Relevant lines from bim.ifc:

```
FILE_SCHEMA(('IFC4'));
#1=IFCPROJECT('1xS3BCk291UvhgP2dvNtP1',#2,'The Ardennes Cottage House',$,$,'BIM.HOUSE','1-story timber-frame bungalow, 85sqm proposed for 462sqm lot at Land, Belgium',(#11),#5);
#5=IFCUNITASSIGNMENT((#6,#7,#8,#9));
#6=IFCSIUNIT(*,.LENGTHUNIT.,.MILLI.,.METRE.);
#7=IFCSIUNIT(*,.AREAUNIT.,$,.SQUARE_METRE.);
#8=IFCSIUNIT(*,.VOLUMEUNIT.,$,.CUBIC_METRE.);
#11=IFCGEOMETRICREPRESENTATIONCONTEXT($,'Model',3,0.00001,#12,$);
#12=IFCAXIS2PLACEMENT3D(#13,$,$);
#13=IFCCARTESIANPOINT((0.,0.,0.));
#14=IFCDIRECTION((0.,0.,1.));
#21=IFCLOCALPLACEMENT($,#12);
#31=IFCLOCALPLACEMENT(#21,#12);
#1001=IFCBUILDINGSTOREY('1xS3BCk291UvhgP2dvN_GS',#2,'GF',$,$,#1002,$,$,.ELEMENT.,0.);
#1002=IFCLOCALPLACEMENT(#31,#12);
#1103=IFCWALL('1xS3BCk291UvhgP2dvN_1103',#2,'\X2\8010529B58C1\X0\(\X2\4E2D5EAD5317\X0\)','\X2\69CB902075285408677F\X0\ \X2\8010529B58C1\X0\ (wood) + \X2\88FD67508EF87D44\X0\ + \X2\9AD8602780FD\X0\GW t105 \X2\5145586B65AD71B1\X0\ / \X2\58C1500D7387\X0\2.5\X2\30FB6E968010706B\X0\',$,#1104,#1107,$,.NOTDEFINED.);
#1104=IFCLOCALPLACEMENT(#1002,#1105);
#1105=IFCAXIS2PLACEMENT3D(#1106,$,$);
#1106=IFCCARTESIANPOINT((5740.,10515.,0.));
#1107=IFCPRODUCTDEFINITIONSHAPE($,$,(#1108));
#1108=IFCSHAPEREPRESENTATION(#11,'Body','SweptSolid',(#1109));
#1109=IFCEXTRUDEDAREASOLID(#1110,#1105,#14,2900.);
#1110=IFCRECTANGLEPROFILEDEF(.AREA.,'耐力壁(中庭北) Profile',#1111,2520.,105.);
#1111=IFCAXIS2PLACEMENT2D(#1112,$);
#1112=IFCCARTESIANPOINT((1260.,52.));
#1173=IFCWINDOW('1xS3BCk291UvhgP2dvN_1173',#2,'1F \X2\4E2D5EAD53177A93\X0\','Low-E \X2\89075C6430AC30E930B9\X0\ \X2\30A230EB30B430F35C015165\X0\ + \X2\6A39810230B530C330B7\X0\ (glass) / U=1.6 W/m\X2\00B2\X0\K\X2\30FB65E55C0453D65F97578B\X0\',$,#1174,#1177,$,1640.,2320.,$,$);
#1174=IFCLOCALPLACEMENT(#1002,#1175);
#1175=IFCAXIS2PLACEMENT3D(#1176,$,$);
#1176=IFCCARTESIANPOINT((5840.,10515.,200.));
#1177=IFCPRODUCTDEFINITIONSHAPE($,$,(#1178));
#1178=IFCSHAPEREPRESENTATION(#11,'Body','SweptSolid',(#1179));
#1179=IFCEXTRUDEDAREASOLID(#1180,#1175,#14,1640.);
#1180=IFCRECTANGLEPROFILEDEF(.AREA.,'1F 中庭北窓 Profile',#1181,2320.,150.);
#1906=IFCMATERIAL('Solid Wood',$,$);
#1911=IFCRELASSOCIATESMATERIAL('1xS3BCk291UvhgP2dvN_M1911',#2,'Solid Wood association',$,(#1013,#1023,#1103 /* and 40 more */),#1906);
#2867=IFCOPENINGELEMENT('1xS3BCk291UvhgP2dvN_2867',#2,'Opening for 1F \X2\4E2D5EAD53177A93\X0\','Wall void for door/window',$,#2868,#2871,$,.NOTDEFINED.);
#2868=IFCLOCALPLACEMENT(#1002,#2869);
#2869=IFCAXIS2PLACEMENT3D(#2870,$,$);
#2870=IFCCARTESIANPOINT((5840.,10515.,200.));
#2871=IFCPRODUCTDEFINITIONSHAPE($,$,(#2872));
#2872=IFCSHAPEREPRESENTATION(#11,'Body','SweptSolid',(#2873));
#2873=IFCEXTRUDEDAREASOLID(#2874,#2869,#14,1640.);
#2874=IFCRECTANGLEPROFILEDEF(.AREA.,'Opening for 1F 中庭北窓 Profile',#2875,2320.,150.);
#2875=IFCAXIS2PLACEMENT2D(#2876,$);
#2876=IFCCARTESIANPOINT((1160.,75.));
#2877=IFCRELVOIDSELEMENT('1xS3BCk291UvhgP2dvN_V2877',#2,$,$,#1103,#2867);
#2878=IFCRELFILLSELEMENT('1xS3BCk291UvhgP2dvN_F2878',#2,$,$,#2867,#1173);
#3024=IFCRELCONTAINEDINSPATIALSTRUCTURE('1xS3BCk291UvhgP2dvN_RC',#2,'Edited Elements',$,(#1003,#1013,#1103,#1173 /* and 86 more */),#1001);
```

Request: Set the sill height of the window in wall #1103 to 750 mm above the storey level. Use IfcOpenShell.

```python
import numpy as np
import ifcopenshell
import ifcopenshell.api.geometry
import ifcopenshell.geom
import ifcopenshell.util.element
import ifcopenshell.util.placement
import ifcopenshell.util.shape
import ifcopenshell.util.unit

model = ifcopenshell.open("bim.ifc")
unit_scale = ifcopenshell.util.unit.calculate_unit_scale(model)

window = model.by_guid("1xS3BCk291UvhgP2dvN_1173")
opening = window.FillsVoids[0].RelatingOpeningElement
storey = ifcopenshell.util.element.get_container(window, ifc_class="IfcBuildingStorey")
level = ifcopenshell.util.placement.get_local_placement(storey.ObjectPlacement)[2, 3]

# The opening's origin need not be at the sill, so measure its lowest point.
shape = ifcopenshell.geom.create_shape(ifcopenshell.geom.settings(), opening)
bottom = ifcopenshell.util.shape.get_shape_bottom_elevation(shape, shape.geometry) / unit_scale
dz = level + 750.0 - bottom

shift = np.array([0.0, 0.0, dz])
# The window is not placed relative to its opening, so move both.
for product in (opening, window):
    matrix = ifcopenshell.util.placement.get_local_placement(product.ObjectPlacement)
    matrix[:3, 3] += shift
    ifcopenshell.api.geometry.edit_object_placement(model, product=product, matrix=matrix, is_si=False)

print(f"moved by {dz * unit_scale:+.3f} m")

model.write("bim_edited.ifc")
```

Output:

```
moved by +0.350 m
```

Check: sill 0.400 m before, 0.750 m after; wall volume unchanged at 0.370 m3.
